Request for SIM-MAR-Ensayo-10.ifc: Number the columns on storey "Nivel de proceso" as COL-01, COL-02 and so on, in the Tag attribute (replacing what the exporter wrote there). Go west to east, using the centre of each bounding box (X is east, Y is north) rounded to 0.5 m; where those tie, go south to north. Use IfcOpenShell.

First a look at what the model holds.

```python
import ifcopenshell
import ifcopenshell.util.element
import ifcopenshell.util.placement

model = ifcopenshell.open("SIM-MAR-Ensayo-10.ifc")
print(model.schema)
storey = next(s for s in model.by_type("IfcBuildingStorey") if s.Name == "Nivel de proceso")
columns = [e for e in ifcopenshell.util.element.get_decomposition(storey) if e.is_a("IfcColumn")]
for e in sorted(columns, key=lambda e: e.id()):
    origin = ifcopenshell.util.placement.get_local_placement(e.ObjectPlacement)[:3, 3]
    print(e.id(), e.Tag, e.Name, origin.round(2) + 0.0, sep=" | ")
```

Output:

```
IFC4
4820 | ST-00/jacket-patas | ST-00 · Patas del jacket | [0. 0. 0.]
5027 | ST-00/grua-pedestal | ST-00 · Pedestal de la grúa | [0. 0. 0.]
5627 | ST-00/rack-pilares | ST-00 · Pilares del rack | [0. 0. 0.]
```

```python
import ifcopenshell
import ifcopenshell.geom
import ifcopenshell.util.element
import ifcopenshell.util.shape

model = ifcopenshell.open("SIM-MAR-Ensayo-10.ifc")
settings = ifcopenshell.geom.settings()
settings.set("use-world-coords", True)


def centre(element):
    shape = ifcopenshell.geom.create_shape(settings, element)
    return ifcopenshell.util.shape.get_bbox_centroid(shape.geometry)


storey = next(s for s in model.by_type("IfcBuildingStorey") if s.Name == "Nivel de proceso")
columns = [e for e in ifcopenshell.util.element.get_decomposition(storey) if e.is_a("IfcColumn")]

# Insertion points can sit at a corner or the storey origin, so sort by the geometry (in metres).
centres = {e: centre(e) for e in columns}
columns.sort(key=lambda e: (round(centres[e][0] / 0.5), centres[e][1]))

for i, e in enumerate(columns, start=1):
    number = f"COL-{i:02d}"
    e.Tag = number
    print(e.id(), number)

model.write("SIM-MAR-Ensayo-10-out.ifc")
```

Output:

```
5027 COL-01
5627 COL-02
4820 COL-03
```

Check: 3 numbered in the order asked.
